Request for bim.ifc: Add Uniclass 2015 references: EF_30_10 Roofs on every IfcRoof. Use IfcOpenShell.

First a look at what the model holds.

```python
import ifcopenshell

model = ifcopenshell.open("bim.ifc")
print(model.schema)
print("classifications:", [c.Name for c in model.by_type("IfcClassification")])
for ifc_class in ("IfcDoor", "IfcRoof", "IfcStair", "IfcWall", "IfcWindow"):
    print(ifc_class, len(model.by_type(ifc_class)))
```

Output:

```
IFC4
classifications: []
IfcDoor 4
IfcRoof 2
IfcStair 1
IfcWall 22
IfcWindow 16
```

```python
import ifcopenshell
import ifcopenshell.api.classification

model = ifcopenshell.open("bim.ifc")

system = ifcopenshell.api.classification.add_classification(model, classification="Uniclass 2015")

codes = {
    "IfcRoof": ("EF_30_10", "Roofs"),
}
for ifc_class, (code, name) in codes.items():
    products = model.by_type(ifc_class)
    ifcopenshell.api.classification.add_reference(
        model, products=products, classification=system, identification=code, name=name
    )
    print(code, len(products))

model.write("bim_rev.ifc")
```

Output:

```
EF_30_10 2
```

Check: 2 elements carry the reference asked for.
